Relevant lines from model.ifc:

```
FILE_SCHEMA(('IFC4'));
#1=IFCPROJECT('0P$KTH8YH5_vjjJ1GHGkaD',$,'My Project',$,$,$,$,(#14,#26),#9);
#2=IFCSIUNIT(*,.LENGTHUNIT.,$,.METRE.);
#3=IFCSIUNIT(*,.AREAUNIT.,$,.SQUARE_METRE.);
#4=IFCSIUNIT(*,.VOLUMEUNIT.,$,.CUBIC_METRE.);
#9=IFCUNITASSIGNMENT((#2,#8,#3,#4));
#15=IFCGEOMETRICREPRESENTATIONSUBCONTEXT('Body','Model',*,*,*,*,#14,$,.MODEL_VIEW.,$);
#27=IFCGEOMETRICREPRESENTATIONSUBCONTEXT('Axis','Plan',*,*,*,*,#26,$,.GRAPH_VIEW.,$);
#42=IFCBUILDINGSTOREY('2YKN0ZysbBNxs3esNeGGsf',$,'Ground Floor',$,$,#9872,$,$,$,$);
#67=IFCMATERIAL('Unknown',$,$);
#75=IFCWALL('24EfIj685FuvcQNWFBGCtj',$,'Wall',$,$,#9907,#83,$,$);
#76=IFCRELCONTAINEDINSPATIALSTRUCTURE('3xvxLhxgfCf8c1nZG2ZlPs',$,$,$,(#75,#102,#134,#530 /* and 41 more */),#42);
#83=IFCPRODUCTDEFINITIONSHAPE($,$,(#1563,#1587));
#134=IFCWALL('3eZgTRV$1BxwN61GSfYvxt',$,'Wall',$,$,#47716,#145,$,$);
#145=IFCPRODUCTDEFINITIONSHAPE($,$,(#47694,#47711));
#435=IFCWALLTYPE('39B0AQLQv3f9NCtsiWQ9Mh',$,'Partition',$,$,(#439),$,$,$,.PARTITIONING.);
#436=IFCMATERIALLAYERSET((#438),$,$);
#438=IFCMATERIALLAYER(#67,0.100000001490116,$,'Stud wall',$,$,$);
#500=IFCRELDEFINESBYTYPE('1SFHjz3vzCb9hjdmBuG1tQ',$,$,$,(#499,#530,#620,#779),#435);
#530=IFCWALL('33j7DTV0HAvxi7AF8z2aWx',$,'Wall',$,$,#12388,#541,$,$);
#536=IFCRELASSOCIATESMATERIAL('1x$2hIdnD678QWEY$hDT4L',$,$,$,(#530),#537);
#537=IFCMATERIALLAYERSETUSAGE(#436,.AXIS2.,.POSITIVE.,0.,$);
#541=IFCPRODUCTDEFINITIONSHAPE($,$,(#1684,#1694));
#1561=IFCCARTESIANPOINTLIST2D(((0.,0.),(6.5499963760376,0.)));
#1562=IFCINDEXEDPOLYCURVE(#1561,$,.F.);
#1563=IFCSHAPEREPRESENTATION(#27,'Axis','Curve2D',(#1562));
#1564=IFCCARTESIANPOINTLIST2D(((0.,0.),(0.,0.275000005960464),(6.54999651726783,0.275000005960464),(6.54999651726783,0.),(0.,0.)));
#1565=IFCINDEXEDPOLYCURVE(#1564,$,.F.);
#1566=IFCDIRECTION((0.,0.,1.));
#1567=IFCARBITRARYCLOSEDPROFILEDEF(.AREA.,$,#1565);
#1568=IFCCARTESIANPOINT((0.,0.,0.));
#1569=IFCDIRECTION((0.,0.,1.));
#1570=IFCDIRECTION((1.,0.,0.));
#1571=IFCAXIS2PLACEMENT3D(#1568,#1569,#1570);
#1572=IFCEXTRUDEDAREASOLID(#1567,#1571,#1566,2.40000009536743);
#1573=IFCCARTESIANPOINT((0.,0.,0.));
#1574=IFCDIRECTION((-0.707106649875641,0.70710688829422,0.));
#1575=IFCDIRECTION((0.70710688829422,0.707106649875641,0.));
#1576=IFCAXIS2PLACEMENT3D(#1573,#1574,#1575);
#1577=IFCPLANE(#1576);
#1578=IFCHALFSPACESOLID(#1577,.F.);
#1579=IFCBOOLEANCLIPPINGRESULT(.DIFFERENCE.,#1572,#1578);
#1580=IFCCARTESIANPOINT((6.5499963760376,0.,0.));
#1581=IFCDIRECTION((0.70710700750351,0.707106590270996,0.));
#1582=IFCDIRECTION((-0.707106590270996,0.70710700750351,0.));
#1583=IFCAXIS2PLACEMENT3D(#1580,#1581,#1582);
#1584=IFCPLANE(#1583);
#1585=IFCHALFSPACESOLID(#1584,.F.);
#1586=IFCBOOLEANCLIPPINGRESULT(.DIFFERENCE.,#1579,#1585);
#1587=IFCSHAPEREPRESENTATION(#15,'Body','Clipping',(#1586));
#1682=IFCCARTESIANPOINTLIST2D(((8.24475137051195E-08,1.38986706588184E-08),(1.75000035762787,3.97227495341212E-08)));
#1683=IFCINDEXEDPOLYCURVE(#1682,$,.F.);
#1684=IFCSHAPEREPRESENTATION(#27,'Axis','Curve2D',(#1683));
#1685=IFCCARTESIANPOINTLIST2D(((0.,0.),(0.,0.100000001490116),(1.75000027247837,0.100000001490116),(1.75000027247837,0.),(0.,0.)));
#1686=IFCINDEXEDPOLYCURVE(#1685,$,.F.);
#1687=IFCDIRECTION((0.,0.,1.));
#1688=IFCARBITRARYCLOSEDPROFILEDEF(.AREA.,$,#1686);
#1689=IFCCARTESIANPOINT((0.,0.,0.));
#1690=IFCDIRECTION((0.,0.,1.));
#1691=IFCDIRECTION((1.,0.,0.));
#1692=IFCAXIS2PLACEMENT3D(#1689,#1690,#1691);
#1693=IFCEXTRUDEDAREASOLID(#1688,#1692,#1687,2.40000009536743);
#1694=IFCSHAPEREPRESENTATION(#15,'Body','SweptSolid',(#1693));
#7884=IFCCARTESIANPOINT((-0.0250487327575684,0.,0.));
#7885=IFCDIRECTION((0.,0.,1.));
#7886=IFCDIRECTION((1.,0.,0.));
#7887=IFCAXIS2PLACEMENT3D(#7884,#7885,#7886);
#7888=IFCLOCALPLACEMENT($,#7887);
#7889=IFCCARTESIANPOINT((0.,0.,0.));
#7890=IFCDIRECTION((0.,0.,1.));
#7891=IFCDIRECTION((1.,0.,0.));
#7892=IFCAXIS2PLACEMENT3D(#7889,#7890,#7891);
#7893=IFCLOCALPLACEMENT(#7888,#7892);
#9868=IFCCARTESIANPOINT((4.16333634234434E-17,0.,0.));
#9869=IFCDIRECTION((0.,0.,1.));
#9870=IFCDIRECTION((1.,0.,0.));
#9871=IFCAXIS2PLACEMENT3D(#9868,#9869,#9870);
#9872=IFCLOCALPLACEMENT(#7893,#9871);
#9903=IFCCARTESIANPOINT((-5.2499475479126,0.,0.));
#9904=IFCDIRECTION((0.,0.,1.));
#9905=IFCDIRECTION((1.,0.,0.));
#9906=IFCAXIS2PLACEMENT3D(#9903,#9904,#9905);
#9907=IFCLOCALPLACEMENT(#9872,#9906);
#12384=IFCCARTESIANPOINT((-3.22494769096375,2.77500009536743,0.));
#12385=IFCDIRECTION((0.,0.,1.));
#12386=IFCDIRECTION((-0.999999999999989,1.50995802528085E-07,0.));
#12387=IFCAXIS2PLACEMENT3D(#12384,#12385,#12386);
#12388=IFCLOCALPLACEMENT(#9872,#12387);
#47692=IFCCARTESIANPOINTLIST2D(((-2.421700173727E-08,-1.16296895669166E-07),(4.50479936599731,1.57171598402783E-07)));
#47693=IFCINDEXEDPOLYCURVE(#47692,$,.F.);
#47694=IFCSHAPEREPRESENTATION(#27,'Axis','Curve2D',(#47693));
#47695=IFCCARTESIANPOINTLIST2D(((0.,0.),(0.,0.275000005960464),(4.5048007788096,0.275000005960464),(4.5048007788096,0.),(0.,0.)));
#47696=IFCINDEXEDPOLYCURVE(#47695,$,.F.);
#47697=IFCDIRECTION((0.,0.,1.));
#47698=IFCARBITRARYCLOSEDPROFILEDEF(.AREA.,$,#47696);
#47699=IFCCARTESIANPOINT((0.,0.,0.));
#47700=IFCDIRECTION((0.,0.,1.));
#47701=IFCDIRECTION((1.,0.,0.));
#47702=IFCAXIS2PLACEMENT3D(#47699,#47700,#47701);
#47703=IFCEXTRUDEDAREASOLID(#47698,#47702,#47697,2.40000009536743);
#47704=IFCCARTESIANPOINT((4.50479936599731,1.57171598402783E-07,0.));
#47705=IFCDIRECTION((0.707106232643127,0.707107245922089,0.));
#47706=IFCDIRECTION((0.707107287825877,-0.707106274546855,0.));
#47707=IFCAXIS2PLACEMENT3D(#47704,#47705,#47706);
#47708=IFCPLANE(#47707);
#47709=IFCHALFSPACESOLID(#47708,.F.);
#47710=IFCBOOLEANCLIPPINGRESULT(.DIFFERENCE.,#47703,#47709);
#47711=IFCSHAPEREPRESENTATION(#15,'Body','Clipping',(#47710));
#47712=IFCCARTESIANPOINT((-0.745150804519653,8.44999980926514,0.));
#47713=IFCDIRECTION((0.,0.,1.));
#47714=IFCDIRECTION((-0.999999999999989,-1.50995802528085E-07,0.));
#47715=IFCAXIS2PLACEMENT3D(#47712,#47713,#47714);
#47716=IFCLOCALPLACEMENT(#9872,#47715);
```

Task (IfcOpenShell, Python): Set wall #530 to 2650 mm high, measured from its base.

```python
import ifcopenshell
import ifcopenshell.geom
import ifcopenshell.util.representation
import ifcopenshell.util.shape
import ifcopenshell.util.unit

model = ifcopenshell.open("model.ifc")
unit_scale = ifcopenshell.util.unit.calculate_unit_scale(model)
settings = ifcopenshell.geom.settings()


def volume(element):
    """Net volume in cubic metres, openings subtracted."""
    shape = ifcopenshell.geom.create_shape(settings, element)
    return ifcopenshell.util.shape.get_volume(shape.geometry)


wall = model.by_guid("33j7DTV0HAvxi7AF8z2aWx")
before = volume(wall)

body = ifcopenshell.util.representation.get_representation(wall, "Model", "Body")
solid = body.Items[0]
old_height = solid.Depth
solid.Depth = 2.65 / unit_scale
after = volume(wall)

print(f"height {old_height:g} -> {solid.Depth:g}, volume {before:.3f} -> {after:.3f} m3")

model.write("model_updated.ifc")
```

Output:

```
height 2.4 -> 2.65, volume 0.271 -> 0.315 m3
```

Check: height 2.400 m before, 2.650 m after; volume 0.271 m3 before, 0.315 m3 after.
